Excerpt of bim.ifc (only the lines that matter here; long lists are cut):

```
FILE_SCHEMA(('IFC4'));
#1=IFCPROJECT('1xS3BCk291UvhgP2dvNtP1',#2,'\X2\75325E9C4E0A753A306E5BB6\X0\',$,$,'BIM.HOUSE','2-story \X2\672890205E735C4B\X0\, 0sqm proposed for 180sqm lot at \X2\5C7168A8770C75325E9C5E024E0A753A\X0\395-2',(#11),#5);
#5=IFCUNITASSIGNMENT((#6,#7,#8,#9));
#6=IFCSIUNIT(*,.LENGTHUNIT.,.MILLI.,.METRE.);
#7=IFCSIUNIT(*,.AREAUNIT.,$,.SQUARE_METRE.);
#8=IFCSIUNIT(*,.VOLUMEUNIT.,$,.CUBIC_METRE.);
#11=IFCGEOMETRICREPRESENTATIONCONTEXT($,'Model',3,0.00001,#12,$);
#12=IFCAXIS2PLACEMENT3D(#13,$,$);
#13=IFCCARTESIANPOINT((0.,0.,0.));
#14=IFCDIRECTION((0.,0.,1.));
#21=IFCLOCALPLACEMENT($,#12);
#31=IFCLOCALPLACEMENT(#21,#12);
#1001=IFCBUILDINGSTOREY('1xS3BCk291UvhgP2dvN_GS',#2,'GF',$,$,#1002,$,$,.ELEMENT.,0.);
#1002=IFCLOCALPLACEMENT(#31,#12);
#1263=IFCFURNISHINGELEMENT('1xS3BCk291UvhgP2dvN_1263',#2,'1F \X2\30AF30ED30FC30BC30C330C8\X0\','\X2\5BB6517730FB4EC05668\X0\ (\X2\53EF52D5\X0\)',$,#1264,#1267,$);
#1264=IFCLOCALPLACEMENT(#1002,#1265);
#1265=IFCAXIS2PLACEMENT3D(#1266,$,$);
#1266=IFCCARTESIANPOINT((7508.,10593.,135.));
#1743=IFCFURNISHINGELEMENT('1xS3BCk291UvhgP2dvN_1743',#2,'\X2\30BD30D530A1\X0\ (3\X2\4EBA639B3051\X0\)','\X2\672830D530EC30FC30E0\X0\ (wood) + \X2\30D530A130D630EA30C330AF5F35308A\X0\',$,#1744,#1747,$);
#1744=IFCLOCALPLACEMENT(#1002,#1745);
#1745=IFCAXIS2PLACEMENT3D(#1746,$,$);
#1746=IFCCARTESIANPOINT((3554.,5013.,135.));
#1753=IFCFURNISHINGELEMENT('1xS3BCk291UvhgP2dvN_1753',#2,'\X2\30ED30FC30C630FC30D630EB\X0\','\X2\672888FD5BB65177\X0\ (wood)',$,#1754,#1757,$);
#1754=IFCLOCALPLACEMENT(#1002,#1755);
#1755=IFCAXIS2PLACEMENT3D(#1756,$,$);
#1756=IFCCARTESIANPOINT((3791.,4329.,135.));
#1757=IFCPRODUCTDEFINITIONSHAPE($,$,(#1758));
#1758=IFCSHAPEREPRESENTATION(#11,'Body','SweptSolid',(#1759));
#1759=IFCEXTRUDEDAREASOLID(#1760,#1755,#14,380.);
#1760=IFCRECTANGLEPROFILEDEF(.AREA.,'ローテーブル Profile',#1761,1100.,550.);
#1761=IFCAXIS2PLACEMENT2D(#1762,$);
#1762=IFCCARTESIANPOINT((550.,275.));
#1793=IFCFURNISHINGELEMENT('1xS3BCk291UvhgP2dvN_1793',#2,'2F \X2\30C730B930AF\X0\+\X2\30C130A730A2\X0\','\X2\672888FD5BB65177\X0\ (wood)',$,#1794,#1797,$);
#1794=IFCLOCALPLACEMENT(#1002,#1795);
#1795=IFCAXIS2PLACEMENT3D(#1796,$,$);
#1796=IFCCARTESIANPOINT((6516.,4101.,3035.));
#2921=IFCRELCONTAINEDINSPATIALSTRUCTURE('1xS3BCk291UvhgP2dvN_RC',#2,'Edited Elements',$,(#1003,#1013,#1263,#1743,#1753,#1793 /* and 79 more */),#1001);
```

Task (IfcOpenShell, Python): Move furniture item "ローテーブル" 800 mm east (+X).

```python
import ifcopenshell
import ifcopenshell.api.geometry
import ifcopenshell.util.placement

model = ifcopenshell.open("bim.ifc")

item = model.by_id(1753)
matrix = ifcopenshell.util.placement.get_local_placement(item.ObjectPlacement)
matrix[0, 3] += 800.0
ifcopenshell.api.geometry.edit_object_placement(model, product=item, matrix=matrix, is_si=False)

print(ifcopenshell.util.placement.get_local_placement(item.ObjectPlacement).round(3) + 0.0)

model.write("bim_rev.ifc")
```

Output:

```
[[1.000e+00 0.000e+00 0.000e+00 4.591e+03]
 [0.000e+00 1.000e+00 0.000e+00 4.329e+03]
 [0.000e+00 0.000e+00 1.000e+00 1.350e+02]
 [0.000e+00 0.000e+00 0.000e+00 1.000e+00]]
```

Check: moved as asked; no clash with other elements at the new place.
